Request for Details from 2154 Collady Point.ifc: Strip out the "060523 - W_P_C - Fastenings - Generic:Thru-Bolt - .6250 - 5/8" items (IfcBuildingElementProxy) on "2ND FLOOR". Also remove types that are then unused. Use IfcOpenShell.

First a look at what the model holds.

```python
import ifcopenshell
import ifcopenshell.util.element

model = ifcopenshell.open("Details from 2154 Collady Point.ifc")
print(model.schema)
storey = next(s for s in model.by_type("IfcBuildingStorey") if s.Name == "2ND FLOOR")
proxies = [e for e in ifcopenshell.util.element.get_decomposition(storey) if e.is_a("IfcBuildingElementProxy")]
seen = {}
for e in proxies:
    element_type = ifcopenshell.util.element.get_type(e)
    name = element_type.Name if element_type not in (None, e) else None
    seen[name] = seen.get(name, 0) + 1
for name, count in sorted(seen.items(), key=str):
    print(count, "x", name)
```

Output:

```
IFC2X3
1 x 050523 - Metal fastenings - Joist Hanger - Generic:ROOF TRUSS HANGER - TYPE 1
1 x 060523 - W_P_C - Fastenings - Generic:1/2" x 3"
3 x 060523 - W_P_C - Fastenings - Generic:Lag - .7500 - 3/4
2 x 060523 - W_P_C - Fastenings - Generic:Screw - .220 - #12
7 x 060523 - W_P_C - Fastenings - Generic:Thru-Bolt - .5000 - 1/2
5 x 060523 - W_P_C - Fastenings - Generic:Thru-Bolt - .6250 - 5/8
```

```python
import ifcopenshell
import ifcopenshell.api.root
import ifcopenshell.util.element

model = ifcopenshell.open("Details from 2154 Collady Point.ifc")

storey = next(s for s in model.by_type("IfcBuildingStorey") if s.Name == "2ND FLOOR")
proxies = [e for e in ifcopenshell.util.element.get_decomposition(storey) if e.is_a("IfcBuildingElementProxy")]
targets = [e for e in proxies if (t := ifcopenshell.util.element.get_type(e)) not in (None, e) and t.Name == "060523 - W_P_C - Fastenings - Generic:Thru-Bolt - .6250 - 5/8"]
types = {ifcopenshell.util.element.get_type(e) for e in targets} - {None, *targets}

for e in targets:
    ifcopenshell.api.root.remove_product(model, product=e)
print(len(targets), "removed")

unused = [t for t in types if not ifcopenshell.util.element.get_types(t)]
for t in unused:
    ifcopenshell.api.root.remove_product(model, product=t)
print(len(unused), "unused types removed")

model.write("Details from 2154 Collady Point_v2.ifc")
```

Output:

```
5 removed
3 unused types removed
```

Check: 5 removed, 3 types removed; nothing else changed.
